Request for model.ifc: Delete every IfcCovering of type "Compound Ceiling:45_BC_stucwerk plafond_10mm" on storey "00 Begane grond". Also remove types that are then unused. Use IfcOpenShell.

First a look at what the model holds.

```python
import ifcopenshell
import ifcopenshell.util.element

model = ifcopenshell.open("model.ifc")
print(model.schema)
storey = next(s for s in model.by_type("IfcBuildingStorey") if s.Name == "00 Begane grond")
coverings = [e for e in ifcopenshell.util.element.get_decomposition(storey) if e.is_a("IfcCovering")]
seen = {}
for e in coverings:
    element_type = ifcopenshell.util.element.get_type(e)
    name = element_type.Name if element_type not in (None, e) else None
    seen[name] = seen.get(name, 0) + 1
for name, count in sorted(seen.items(), key=str):
    print(count, "x", name)
```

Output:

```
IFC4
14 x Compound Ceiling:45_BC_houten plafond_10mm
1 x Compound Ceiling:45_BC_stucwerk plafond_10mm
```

```python
import ifcopenshell
import ifcopenshell.api.root
import ifcopenshell.util.element

model = ifcopenshell.open("model.ifc")

storey = next(s for s in model.by_type("IfcBuildingStorey") if s.Name == "00 Begane grond")
coverings = [e for e in ifcopenshell.util.element.get_decomposition(storey) if e.is_a("IfcCovering")]
targets = [e for e in coverings if (t := ifcopenshell.util.element.get_type(e)) not in (None, e) and t.Name == "Compound Ceiling:45_BC_stucwerk plafond_10mm"]
types = {ifcopenshell.util.element.get_type(e) for e in targets} - {None, *targets}

for e in targets:
    ifcopenshell.api.root.remove_product(model, product=e)
print(len(targets), "removed")

unused = [t for t in types if not ifcopenshell.util.element.get_types(t)]
for t in unused:
    ifcopenshell.api.root.remove_product(model, product=t)
print(len(unused), "unused types removed")

model.write("model_rev.ifc")
```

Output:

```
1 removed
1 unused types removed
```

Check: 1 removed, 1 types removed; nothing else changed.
